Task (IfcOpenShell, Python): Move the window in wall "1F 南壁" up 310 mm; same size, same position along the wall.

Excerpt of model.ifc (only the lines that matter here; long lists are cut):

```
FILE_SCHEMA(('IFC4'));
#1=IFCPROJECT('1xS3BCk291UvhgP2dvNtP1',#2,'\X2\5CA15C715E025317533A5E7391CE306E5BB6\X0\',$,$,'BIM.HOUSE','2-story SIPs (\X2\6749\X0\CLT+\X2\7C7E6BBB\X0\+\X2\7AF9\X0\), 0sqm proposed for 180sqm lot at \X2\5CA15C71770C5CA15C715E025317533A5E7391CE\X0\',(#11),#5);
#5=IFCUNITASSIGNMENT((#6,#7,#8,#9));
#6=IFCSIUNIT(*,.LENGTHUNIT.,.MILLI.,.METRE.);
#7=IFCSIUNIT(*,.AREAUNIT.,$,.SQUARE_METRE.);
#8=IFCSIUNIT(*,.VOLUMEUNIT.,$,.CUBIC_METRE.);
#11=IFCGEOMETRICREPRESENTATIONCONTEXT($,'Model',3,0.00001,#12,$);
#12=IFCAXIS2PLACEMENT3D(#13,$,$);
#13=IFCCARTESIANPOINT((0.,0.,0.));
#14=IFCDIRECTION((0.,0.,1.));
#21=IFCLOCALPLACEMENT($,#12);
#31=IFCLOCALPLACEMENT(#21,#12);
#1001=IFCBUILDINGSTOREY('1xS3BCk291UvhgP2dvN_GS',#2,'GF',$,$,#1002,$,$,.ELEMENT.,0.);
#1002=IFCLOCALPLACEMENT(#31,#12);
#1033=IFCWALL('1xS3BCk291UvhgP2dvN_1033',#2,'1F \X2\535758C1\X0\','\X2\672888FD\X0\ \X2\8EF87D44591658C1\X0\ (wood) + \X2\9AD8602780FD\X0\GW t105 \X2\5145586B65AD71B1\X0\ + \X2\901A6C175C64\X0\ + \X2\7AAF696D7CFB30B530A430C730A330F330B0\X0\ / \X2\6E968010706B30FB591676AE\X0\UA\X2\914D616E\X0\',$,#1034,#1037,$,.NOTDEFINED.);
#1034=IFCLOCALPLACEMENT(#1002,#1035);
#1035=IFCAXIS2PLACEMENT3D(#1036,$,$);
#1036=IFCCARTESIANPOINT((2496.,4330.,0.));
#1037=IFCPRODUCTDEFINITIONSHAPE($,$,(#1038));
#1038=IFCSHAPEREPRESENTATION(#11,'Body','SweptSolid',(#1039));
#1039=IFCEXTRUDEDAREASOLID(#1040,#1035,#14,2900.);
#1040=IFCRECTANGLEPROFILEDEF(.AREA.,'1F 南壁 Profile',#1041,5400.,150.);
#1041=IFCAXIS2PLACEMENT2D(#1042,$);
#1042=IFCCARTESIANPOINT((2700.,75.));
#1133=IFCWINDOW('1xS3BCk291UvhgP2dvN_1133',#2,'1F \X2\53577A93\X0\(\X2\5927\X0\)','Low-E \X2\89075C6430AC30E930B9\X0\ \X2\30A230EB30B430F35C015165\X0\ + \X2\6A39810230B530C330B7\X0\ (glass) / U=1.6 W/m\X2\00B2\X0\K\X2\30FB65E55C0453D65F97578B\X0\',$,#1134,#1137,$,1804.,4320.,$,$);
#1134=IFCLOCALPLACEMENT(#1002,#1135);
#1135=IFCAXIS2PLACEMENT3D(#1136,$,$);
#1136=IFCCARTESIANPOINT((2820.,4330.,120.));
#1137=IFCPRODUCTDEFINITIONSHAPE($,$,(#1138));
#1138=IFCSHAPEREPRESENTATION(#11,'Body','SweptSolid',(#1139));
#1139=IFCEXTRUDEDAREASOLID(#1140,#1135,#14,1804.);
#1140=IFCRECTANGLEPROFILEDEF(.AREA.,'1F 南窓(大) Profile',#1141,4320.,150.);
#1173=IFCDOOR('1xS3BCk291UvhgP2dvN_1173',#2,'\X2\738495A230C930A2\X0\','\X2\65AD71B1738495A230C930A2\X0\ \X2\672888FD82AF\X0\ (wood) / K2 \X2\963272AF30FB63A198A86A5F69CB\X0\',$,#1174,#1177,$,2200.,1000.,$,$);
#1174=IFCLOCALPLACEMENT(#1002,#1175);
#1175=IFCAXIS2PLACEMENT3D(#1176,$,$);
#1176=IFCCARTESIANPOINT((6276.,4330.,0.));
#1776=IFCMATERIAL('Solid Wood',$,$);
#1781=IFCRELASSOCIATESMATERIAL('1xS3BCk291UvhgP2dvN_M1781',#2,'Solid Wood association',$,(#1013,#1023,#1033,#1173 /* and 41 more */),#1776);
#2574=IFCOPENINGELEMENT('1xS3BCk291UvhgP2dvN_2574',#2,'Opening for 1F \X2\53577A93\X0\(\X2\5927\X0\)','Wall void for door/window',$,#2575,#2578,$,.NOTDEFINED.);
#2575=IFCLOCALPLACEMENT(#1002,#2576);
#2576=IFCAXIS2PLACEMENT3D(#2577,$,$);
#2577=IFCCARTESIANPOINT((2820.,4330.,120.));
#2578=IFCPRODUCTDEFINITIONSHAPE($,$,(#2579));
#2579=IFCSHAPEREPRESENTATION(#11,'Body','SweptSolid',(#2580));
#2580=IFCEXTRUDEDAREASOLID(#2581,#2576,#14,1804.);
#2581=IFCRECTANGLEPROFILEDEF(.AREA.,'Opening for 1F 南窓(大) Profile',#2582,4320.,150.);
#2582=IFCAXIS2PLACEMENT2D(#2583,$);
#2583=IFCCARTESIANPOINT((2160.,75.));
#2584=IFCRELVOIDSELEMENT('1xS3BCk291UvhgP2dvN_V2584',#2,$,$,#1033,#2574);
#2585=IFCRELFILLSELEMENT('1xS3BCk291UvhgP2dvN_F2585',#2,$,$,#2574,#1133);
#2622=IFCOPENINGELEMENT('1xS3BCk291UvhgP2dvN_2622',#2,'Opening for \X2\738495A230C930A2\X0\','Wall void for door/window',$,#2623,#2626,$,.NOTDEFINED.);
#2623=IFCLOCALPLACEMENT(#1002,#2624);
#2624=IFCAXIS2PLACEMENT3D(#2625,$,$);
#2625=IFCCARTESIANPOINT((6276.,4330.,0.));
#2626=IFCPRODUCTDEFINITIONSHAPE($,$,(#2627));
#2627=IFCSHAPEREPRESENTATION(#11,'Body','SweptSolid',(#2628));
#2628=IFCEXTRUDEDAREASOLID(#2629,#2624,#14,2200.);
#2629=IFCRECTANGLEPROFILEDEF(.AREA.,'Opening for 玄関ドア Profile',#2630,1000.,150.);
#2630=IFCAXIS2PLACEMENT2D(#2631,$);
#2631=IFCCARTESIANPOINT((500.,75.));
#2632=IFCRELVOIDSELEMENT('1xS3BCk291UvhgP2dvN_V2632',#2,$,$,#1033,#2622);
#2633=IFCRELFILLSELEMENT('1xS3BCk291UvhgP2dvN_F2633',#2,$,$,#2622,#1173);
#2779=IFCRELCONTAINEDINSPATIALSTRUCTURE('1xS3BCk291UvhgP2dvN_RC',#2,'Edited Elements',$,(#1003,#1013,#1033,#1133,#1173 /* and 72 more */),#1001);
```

```python
import numpy as np
import ifcopenshell
import ifcopenshell.api.geometry
import ifcopenshell.util.placement
import ifcopenshell.util.unit

model = ifcopenshell.open("model.ifc")
unit_scale = ifcopenshell.util.unit.calculate_unit_scale(model)

window = model.by_guid("1xS3BCk291UvhgP2dvN_1133")
opening = window.FillsVoids[0].RelatingOpeningElement
dz = 0.31 / unit_scale

shift = np.array([0.0, 0.0, dz])
# The window is not placed relative to its opening, so move both.
for product in (opening, window):
    matrix = ifcopenshell.util.placement.get_local_placement(product.ObjectPlacement)
    matrix[:3, 3] += shift
    ifcopenshell.api.geometry.edit_object_placement(model, product=product, matrix=matrix, is_si=False)

print(f"moved by {dz * unit_scale:+.3f} m")

model.write("model_rev.ifc")
```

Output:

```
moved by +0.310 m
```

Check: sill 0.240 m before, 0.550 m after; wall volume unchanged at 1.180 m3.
